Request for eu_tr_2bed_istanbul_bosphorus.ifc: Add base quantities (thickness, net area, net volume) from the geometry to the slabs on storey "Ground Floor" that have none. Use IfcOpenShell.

First a look at what the model holds.

```python
import ifcopenshell
import ifcopenshell.util.element
import ifcopenshell.util.unit

model = ifcopenshell.open("eu_tr_2bed_istanbul_bosphorus.ifc")
print(model.schema)
for unit_type in ("LENGTHUNIT", "AREAUNIT", "VOLUMEUNIT"):
    print(unit_type, ifcopenshell.util.unit.calculate_unit_scale(model, unit_type))
storey = next(s for s in model.by_type("IfcBuildingStorey") if s.Name == "Ground Floor")
slabs = [e for e in ifcopenshell.util.element.get_decomposition(storey) if e.is_a("IfcSlab")]
for e in sorted(slabs, key=lambda e: e.id()):
    print(e.id(), e.is_a(), e.Name, list(ifcopenshell.util.element.get_psets(e, qtos_only=True)), sep=" | ")
```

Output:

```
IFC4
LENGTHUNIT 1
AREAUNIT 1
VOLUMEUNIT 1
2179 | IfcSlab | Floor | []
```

```python
import ifcopenshell
import ifcopenshell.api.pset
import ifcopenshell.geom
import ifcopenshell.util.element
import ifcopenshell.util.shape
import ifcopenshell.util.unit

model = ifcopenshell.open("eu_tr_2bed_istanbul_bosphorus.ifc")
unit_scale = ifcopenshell.util.unit.calculate_unit_scale(model)
area_scale = ifcopenshell.util.unit.calculate_unit_scale(model, "AREAUNIT")
volume_scale = ifcopenshell.util.unit.calculate_unit_scale(model, "VOLUMEUNIT")
settings = ifcopenshell.geom.settings()

storey = next(s for s in model.by_type("IfcBuildingStorey") if s.Name == "Ground Floor")
slabs = [e for e in ifcopenshell.util.element.get_decomposition(storey) if e.is_a("IfcSlab")]

for e in sorted(slabs, key=lambda e: e.id()):
    if ifcopenshell.util.element.get_psets(e, qtos_only=True, should_inherit=False):
        continue
    # Geometry comes back in metres, in the element's own axes.
    shape = ifcopenshell.geom.create_shape(settings, e)
    values = {
        "Width": ifcopenshell.util.shape.get_z(shape.geometry) / unit_scale,
        "NetArea": ifcopenshell.util.shape.get_footprint_area(shape.geometry) / area_scale,
        "NetVolume": ifcopenshell.util.shape.get_volume(shape.geometry) / volume_scale,
    }
    qto = ifcopenshell.api.pset.add_qto(model, product=e, name="Qto_SlabBaseQuantities")
    ifcopenshell.api.pset.edit_qto(model, qto=qto, properties=values)
    print(e.id(), {k: round(v, 3) for k, v in values.items()})

model.write("eu_tr_2bed_istanbul_bosphorus_updated.ifc")
```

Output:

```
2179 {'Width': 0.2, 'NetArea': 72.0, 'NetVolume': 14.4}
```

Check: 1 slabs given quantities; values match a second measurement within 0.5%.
